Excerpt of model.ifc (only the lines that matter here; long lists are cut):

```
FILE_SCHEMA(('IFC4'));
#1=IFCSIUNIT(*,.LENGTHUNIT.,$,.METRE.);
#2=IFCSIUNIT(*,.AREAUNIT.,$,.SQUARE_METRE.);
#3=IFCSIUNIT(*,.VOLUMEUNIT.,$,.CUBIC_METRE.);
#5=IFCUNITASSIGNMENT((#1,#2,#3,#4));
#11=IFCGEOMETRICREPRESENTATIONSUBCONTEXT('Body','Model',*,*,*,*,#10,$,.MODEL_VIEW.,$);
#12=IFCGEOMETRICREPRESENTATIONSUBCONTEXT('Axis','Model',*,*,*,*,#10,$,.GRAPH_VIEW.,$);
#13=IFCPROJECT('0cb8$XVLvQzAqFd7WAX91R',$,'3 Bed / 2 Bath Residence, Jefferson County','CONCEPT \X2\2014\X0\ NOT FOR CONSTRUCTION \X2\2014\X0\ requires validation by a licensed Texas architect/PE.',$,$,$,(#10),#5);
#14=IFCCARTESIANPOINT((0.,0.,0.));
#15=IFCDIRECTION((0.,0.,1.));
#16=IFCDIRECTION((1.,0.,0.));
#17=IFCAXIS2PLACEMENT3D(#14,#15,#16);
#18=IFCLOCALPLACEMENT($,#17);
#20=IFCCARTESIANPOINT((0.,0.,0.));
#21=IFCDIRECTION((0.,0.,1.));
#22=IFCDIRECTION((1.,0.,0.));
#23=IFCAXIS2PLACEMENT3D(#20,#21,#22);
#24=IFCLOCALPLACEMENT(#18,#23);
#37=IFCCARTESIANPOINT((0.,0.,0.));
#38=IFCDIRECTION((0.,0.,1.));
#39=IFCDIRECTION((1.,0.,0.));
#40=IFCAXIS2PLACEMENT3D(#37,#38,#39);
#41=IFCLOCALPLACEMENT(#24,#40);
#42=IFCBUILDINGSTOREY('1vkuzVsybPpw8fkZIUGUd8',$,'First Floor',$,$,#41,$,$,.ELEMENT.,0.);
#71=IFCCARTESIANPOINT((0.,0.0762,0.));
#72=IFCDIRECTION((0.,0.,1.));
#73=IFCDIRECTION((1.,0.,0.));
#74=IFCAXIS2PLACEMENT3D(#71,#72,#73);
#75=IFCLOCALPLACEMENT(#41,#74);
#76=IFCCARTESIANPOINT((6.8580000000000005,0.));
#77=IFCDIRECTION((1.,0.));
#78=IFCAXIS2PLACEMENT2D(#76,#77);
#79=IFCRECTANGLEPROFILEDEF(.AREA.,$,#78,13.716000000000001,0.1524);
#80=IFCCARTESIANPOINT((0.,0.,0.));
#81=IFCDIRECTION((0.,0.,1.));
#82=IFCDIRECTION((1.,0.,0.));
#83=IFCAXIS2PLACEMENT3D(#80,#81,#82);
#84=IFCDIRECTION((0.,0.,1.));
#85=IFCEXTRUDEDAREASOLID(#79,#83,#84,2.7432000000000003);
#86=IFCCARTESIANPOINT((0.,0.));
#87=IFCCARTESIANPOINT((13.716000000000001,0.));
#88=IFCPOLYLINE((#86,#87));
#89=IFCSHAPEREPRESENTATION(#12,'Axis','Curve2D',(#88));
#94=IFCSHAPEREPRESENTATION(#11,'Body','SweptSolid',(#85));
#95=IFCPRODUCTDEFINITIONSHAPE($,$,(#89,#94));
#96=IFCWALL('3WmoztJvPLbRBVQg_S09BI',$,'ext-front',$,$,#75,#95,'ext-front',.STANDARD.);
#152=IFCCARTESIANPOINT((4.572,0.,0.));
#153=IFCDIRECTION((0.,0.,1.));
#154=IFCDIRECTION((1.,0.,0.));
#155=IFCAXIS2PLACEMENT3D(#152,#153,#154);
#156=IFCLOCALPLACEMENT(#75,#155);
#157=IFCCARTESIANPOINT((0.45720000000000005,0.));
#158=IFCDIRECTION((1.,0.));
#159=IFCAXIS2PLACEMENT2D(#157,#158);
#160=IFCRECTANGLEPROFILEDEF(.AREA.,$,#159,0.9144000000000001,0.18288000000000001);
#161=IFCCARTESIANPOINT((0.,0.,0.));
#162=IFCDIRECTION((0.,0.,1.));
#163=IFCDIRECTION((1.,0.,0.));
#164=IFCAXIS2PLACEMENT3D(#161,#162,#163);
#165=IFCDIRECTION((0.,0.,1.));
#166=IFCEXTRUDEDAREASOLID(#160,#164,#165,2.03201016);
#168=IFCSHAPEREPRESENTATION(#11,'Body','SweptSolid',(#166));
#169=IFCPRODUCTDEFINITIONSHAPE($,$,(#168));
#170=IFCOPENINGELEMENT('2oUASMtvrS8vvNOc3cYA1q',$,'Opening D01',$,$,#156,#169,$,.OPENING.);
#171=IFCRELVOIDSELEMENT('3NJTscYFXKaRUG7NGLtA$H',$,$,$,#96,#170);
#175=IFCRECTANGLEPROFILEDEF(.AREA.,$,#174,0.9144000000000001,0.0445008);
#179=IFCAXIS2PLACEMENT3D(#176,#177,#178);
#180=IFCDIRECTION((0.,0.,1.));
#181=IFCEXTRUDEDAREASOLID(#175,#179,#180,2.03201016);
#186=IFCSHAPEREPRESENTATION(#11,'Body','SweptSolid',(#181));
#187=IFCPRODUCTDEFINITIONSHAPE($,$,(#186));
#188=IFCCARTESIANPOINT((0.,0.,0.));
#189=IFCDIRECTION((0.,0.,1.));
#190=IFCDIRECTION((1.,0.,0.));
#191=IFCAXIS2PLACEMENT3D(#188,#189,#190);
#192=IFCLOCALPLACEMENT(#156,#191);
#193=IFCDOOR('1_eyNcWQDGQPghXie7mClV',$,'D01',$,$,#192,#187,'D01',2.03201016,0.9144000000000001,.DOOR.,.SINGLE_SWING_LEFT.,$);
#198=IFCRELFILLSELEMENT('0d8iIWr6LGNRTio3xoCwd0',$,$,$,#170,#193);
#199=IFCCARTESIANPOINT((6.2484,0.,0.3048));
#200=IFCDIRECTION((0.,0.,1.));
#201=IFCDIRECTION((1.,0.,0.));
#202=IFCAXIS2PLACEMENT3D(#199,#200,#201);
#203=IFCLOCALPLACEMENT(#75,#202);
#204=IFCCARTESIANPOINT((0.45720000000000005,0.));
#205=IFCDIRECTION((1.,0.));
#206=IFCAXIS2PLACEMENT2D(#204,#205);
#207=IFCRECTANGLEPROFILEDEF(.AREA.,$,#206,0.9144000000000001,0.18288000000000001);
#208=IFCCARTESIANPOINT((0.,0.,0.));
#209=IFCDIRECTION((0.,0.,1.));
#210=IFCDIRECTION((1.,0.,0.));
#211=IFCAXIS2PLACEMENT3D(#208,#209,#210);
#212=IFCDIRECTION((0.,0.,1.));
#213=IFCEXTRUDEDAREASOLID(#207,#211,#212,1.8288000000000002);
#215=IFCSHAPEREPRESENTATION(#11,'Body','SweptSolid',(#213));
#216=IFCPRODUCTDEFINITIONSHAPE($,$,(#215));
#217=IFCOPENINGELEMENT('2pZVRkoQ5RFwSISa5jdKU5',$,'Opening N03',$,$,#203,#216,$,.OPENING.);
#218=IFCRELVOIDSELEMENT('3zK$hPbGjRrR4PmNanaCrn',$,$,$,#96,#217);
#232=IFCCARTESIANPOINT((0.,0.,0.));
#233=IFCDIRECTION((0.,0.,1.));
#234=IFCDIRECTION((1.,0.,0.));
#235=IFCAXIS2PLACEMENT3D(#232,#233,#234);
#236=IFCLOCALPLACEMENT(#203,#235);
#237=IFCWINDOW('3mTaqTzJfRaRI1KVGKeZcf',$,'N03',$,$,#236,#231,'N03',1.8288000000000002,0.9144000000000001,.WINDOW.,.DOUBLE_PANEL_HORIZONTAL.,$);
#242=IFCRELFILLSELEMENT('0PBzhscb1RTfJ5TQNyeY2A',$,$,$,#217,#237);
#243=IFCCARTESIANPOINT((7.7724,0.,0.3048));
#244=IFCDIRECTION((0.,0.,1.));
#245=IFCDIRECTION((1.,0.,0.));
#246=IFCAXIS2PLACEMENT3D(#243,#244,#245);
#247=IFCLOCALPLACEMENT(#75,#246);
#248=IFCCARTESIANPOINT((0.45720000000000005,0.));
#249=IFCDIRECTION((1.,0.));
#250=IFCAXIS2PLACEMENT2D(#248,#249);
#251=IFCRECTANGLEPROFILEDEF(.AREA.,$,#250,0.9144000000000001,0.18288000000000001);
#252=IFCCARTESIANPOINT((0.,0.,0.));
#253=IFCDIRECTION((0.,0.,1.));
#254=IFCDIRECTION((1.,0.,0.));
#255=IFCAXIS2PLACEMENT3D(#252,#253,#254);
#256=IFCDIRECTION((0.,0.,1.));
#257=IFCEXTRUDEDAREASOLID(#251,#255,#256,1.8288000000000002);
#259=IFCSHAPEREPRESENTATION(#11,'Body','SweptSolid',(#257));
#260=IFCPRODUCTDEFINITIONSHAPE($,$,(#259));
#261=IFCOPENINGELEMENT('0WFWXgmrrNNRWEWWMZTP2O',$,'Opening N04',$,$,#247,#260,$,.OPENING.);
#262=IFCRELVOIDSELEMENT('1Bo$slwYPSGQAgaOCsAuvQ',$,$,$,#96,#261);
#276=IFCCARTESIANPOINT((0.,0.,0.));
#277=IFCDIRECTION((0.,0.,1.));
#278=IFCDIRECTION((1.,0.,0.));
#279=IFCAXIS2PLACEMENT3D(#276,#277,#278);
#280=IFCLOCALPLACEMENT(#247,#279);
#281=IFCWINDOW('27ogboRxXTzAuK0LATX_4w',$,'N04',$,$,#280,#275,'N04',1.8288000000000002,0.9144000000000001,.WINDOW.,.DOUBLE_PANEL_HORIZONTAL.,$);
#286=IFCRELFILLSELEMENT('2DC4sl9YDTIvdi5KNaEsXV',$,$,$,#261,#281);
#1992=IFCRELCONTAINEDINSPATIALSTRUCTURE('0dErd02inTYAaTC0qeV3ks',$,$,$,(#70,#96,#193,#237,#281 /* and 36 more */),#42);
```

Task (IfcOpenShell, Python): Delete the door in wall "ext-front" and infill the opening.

```python
import ifcopenshell
import ifcopenshell.api.feature
import ifcopenshell.api.root
import ifcopenshell.geom
import ifcopenshell.util.shape

model = ifcopenshell.open("model.ifc")
settings = ifcopenshell.geom.settings()


def volume(element):
    """Net volume in cubic metres, openings subtracted."""
    shape = ifcopenshell.geom.create_shape(settings, element)
    return ifcopenshell.util.shape.get_volume(shape.geometry)


door = model.by_guid("1_eyNcWQDGQPghXie7mClV")
opening = door.FillsVoids[0].RelatingOpeningElement
wall = opening.VoidsElements[0].RelatingBuildingElement
before = volume(wall)

ifcopenshell.api.root.remove_product(model, product=door)
ifcopenshell.api.feature.remove_feature(model, feature=opening)

after = volume(wall)

print(f"wall volume {before:.3f} -> {after:.3f} m3")

model.write("model-out.ifc")
```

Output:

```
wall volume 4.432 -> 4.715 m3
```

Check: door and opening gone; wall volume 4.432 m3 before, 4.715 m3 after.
